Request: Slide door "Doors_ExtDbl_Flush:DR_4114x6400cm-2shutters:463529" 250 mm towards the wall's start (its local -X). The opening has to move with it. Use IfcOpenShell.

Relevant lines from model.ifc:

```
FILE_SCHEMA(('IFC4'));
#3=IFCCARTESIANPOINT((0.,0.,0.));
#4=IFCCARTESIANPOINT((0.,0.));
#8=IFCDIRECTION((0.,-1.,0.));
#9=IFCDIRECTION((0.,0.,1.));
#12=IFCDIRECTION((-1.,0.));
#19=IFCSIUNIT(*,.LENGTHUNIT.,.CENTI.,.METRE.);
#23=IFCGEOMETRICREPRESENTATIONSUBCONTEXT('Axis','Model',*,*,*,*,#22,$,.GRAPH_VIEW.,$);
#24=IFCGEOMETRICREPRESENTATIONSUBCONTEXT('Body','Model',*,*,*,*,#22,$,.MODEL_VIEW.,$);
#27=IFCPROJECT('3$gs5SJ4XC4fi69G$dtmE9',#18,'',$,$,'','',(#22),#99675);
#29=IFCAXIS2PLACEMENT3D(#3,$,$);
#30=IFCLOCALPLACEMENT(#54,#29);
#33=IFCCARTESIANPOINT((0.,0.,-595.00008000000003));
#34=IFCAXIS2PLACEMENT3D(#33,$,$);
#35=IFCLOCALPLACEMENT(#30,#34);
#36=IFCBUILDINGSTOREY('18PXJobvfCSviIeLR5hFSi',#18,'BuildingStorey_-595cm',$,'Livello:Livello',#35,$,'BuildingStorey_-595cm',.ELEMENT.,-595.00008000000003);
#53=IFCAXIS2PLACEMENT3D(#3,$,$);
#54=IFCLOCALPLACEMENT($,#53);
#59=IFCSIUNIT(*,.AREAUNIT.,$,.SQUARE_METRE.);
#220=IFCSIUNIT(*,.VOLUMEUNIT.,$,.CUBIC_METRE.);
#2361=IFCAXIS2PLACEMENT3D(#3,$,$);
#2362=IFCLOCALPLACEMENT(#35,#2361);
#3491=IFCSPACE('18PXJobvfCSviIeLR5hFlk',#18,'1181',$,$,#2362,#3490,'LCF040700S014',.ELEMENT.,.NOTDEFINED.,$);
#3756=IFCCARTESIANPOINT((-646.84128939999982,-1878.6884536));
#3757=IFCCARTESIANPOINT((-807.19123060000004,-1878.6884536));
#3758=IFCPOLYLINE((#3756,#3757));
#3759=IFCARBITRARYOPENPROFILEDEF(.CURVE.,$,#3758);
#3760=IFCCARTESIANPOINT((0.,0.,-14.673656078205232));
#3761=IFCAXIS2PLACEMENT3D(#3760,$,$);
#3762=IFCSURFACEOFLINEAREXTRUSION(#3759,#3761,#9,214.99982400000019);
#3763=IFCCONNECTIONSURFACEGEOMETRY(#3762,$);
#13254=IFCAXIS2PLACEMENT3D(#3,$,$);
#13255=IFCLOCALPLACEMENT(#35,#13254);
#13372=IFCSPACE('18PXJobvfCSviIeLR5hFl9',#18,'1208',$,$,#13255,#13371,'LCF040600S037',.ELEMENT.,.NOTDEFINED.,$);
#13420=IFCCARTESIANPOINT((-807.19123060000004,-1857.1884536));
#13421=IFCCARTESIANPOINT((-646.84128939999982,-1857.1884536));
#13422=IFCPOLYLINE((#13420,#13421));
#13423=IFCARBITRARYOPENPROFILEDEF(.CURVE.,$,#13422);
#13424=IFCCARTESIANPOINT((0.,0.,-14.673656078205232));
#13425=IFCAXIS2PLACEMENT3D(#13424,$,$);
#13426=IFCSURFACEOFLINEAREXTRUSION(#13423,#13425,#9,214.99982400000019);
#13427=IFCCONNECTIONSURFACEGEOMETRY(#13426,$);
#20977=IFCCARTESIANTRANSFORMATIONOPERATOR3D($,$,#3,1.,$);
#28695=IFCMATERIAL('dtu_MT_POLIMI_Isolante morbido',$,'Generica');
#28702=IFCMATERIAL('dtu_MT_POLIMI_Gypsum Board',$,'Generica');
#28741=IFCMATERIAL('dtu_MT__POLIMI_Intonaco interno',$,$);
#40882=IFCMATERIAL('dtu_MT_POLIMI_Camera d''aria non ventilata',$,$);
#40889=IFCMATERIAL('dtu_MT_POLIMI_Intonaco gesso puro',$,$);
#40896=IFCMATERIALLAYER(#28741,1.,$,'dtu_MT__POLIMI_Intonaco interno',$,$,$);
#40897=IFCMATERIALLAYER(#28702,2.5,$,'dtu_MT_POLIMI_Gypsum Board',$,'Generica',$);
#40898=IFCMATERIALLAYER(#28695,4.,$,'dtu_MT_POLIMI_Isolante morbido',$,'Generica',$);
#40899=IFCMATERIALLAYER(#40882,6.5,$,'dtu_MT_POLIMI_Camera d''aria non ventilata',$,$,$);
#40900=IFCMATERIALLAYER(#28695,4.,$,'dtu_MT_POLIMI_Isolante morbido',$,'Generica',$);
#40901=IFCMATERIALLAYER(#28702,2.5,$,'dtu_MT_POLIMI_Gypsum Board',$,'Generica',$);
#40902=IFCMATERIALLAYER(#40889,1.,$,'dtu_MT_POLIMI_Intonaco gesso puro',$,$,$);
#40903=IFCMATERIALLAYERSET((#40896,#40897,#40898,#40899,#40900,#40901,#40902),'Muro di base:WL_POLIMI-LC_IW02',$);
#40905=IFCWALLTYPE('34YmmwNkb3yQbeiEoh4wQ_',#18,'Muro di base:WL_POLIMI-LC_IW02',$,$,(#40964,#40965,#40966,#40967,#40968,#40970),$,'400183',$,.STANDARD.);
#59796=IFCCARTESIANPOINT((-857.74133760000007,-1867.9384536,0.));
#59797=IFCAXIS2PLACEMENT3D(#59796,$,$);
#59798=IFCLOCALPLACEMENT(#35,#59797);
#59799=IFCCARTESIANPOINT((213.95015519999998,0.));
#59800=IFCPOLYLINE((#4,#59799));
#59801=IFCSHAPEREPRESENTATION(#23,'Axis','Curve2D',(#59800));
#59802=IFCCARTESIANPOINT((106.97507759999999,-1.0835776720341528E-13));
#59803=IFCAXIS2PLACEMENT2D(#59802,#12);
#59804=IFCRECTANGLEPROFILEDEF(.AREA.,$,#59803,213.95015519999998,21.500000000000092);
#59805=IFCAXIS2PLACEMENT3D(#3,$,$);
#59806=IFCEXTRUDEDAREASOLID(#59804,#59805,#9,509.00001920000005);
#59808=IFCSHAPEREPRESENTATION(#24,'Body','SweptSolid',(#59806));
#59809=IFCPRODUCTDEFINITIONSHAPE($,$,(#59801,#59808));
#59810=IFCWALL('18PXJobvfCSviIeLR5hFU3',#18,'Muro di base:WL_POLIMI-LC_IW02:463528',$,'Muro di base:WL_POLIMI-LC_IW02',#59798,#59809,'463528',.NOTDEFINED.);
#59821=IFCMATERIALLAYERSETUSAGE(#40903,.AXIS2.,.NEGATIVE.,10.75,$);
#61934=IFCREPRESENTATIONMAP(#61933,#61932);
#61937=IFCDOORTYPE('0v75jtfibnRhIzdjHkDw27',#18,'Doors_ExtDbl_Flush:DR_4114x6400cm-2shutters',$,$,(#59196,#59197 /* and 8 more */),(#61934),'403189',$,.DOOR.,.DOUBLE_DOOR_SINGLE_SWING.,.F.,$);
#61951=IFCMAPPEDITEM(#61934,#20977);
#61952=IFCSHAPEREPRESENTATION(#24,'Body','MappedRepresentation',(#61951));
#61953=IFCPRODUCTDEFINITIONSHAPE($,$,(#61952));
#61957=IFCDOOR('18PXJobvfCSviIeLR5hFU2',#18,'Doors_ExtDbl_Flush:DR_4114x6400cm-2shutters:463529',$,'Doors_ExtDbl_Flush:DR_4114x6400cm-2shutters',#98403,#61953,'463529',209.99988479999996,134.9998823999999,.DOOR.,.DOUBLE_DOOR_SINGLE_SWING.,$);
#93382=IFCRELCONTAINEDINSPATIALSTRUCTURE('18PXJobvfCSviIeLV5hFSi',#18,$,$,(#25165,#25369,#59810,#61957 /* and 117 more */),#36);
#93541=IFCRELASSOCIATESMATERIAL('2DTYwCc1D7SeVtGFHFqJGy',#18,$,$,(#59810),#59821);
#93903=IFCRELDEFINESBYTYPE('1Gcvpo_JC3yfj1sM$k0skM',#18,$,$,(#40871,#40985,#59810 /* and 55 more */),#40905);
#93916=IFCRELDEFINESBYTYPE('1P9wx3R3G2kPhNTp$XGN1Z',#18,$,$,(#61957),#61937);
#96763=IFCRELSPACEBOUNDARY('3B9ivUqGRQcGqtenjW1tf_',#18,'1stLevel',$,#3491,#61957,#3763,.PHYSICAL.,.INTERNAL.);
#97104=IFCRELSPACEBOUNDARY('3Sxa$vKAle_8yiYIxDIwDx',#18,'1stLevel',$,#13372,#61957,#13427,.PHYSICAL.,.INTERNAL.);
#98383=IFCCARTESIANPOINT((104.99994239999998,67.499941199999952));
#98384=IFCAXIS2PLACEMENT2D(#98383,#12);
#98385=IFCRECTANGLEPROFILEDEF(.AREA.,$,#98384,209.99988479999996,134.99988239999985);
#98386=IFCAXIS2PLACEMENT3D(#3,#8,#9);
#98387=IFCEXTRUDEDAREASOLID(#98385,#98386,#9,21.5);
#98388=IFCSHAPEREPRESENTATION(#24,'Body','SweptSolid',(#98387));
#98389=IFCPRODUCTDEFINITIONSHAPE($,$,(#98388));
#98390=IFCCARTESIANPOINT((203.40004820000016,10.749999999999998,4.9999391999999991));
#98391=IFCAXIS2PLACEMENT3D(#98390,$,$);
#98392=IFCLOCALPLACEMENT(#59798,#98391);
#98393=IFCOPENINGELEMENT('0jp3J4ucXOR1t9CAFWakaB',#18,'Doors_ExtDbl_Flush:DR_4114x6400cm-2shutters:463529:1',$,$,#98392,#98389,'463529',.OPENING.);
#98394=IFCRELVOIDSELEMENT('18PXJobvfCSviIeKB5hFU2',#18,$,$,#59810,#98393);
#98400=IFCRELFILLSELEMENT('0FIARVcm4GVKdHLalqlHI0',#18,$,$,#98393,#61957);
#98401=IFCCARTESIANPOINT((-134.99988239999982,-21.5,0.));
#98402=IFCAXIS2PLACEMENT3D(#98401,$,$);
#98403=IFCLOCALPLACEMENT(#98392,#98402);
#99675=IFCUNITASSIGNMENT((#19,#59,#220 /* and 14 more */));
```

```python
import numpy as np
import ifcopenshell
import ifcopenshell.api.geometry
import ifcopenshell.util.placement
import ifcopenshell.util.unit

model = ifcopenshell.open("model.ifc")
unit_scale = ifcopenshell.util.unit.calculate_unit_scale(model)

door = model.by_guid("18PXJobvfCSviIeLR5hFU2")
opening = door.FillsVoids[0].RelatingOpeningElement
wall = opening.VoidsElements[0].RelatingBuildingElement

wall_matrix = ifcopenshell.util.placement.get_local_placement(wall.ObjectPlacement)
shift = wall_matrix[:3, 0] * -0.25 / unit_scale
before = ifcopenshell.util.placement.get_local_placement(door.ObjectPlacement)[:3, 3].copy()

# The door is placed relative to its opening, so it follows when the opening moves.
matrix = ifcopenshell.util.placement.get_local_placement(opening.ObjectPlacement)
matrix[:3, 3] += shift
ifcopenshell.api.geometry.edit_object_placement(
    model, product=opening, matrix=matrix, is_si=False, should_transform_children=True
)

# Space boundary surfaces are stored in each space's coordinates; move them too.
for rel in door.ProvidesBoundaries:
    if not rel.ConnectionGeometry:
        continue
    surface = rel.ConnectionGeometry.SurfaceOnRelatingElement
    space_matrix = ifcopenshell.util.placement.get_local_placement(rel.RelatingSpace.ObjectPlacement)
    point = np.array(surface.Position.Location.Coordinates) + space_matrix[:3, :3].T @ shift
    surface.Position = model.createIfcAxis2Placement3D(
        model.createIfcCartesianPoint(point.tolist()), surface.Position.Axis, surface.Position.RefDirection
    )

after = ifcopenshell.util.placement.get_local_placement(door.ObjectPlacement)[:3, 3]
print("door moved by", (after - before).round(3) + 0.0)

model.write("model_rev.ifc")
```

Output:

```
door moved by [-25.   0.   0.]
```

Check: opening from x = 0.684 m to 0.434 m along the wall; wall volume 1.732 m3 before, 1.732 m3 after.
